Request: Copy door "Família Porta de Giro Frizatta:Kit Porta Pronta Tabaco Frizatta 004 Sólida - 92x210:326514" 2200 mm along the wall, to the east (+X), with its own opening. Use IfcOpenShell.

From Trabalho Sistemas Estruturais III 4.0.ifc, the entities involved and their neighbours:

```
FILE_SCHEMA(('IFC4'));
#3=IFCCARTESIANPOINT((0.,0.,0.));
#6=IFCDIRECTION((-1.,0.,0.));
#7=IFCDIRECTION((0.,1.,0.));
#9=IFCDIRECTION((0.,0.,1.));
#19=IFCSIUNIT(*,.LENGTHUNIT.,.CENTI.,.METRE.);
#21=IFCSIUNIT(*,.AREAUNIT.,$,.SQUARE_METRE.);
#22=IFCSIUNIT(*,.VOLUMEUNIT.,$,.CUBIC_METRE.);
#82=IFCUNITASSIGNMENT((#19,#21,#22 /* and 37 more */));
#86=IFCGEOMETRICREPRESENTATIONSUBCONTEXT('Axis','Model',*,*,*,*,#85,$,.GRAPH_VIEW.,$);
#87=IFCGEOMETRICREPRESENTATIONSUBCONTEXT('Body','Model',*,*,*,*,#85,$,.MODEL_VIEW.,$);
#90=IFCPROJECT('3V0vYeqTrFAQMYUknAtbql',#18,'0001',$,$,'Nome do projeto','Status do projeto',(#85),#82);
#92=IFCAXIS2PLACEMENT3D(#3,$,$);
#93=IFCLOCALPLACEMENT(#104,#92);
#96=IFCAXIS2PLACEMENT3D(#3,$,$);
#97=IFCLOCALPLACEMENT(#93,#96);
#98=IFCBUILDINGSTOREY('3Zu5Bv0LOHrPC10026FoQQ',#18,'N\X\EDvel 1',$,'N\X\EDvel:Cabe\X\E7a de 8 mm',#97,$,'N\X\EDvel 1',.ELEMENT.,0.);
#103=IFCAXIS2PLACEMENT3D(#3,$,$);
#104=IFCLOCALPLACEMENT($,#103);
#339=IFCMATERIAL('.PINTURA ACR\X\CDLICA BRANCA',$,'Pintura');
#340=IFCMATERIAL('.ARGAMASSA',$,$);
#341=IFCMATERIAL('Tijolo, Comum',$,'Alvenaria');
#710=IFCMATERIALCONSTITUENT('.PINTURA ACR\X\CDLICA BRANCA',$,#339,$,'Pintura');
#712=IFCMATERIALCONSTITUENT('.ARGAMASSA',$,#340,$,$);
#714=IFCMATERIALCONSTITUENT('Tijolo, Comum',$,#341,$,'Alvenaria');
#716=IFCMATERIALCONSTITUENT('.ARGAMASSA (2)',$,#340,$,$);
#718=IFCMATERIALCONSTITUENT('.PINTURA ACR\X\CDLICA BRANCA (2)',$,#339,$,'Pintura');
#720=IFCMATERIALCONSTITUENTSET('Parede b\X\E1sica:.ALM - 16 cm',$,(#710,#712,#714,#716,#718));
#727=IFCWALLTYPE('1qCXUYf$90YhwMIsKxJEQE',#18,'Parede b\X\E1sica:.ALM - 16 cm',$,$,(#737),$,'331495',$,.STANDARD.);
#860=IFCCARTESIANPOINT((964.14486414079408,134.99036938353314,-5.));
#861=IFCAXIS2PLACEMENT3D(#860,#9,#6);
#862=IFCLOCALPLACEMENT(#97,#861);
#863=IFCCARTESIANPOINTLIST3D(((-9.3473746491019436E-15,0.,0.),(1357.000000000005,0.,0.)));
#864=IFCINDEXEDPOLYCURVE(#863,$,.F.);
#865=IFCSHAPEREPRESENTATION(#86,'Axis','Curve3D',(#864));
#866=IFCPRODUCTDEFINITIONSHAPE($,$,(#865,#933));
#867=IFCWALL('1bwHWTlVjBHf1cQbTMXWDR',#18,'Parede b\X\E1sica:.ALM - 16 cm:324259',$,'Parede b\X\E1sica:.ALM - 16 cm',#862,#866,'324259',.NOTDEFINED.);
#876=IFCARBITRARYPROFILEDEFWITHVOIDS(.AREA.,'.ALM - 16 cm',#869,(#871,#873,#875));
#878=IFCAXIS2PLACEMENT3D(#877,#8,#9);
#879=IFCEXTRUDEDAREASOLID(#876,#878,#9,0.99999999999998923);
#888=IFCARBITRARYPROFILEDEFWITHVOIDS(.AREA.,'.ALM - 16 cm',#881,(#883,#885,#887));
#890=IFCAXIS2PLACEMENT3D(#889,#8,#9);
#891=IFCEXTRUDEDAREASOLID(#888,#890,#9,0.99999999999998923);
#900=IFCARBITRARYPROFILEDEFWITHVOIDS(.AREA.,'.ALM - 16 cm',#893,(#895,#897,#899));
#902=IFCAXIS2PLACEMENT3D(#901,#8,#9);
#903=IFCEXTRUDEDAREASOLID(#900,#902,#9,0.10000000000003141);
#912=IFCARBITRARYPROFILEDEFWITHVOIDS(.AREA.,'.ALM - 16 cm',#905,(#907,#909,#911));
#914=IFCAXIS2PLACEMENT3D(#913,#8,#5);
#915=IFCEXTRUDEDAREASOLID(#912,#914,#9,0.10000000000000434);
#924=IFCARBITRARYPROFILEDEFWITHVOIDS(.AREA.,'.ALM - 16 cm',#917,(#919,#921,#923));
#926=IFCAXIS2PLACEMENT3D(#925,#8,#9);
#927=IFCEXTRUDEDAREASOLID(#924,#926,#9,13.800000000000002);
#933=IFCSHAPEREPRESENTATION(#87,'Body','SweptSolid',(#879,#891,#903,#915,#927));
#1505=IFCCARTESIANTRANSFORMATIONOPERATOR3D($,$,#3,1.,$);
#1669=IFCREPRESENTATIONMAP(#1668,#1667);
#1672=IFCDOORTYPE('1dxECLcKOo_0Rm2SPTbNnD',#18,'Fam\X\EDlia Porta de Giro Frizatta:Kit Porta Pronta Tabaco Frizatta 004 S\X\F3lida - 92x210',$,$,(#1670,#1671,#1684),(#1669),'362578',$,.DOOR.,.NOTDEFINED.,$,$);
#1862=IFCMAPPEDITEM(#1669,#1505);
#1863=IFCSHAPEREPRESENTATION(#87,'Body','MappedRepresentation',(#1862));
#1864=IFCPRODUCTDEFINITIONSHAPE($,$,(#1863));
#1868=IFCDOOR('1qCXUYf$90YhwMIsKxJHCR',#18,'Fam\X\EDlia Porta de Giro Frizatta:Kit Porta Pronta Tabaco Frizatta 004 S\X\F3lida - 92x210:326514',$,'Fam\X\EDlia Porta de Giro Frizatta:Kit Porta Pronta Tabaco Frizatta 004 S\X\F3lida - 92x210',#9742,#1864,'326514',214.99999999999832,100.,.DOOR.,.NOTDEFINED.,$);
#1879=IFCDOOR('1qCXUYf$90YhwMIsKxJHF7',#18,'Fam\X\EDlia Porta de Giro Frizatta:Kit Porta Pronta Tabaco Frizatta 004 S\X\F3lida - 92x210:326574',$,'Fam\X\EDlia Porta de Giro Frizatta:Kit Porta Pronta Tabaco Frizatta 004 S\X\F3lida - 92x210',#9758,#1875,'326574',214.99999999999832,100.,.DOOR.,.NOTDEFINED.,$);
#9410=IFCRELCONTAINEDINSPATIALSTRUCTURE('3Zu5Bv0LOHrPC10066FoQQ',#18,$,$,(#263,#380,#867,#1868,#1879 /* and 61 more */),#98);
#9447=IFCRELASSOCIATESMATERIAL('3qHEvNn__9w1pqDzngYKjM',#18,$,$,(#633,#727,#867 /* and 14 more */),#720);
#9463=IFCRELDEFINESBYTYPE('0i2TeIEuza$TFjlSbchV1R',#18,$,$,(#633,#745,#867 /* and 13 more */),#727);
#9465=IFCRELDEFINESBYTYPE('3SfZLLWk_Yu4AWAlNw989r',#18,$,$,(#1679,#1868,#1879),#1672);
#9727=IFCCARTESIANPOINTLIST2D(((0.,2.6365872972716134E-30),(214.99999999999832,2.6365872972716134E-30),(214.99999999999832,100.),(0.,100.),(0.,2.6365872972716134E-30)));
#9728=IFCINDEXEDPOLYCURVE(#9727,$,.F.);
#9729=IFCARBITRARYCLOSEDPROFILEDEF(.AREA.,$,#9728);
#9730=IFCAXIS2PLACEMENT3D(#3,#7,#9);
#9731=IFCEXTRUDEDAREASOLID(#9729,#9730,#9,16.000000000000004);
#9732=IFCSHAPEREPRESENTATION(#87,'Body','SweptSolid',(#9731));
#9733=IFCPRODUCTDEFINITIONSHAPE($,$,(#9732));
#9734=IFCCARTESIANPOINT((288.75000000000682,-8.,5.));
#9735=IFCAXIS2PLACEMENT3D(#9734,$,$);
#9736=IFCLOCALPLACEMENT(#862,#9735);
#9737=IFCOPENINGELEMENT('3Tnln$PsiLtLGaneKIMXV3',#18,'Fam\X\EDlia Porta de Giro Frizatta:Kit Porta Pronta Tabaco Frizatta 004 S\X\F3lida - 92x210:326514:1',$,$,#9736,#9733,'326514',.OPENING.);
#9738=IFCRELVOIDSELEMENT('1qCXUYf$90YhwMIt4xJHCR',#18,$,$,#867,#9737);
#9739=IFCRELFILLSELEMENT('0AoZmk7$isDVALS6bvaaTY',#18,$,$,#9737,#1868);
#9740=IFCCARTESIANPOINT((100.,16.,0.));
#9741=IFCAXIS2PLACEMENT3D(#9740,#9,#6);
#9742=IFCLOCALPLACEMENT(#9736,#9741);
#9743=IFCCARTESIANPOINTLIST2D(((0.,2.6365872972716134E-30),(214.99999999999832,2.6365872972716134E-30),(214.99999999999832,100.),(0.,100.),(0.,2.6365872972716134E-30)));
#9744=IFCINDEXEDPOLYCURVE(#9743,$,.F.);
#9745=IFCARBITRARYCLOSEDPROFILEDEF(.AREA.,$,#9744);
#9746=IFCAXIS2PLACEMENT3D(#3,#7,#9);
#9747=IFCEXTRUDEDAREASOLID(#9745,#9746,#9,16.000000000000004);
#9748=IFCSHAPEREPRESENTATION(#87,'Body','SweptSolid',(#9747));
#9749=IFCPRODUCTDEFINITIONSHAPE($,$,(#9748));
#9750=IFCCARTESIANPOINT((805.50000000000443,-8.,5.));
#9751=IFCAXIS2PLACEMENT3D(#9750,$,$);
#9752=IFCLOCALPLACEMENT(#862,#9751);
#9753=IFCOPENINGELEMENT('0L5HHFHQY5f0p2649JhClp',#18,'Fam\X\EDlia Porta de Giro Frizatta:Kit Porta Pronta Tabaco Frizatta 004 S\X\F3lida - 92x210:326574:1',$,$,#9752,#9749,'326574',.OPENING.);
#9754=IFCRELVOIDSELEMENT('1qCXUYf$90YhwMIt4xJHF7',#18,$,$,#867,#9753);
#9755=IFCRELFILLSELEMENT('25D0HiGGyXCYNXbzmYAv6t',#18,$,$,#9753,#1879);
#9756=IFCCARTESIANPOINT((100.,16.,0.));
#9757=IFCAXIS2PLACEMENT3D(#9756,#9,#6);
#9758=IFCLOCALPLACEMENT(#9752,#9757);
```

```python
import ifcopenshell
import ifcopenshell.api.feature
import ifcopenshell.api.geometry
import ifcopenshell.api.root
import ifcopenshell.geom
import ifcopenshell.util.element
import ifcopenshell.util.placement
import ifcopenshell.util.shape
import ifcopenshell.util.unit

model = ifcopenshell.open("Trabalho Sistemas Estruturais III 4.0.ifc")
unit_scale = ifcopenshell.util.unit.calculate_unit_scale(model)
settings = ifcopenshell.geom.settings()


def volume(element):
    """Net volume in cubic metres, openings subtracted."""
    shape = ifcopenshell.geom.create_shape(settings, element)
    return ifcopenshell.util.shape.get_volume(shape.geometry)


def reuse_history(source, copy):
    """copy_class also copies each property set's owner history, people and application; keep the originals."""
    for rel in copy.IsDefinedBy:
        if rel.is_a("IfcRelDefinesByProperties") and (history := rel.RelatingPropertyDefinition.OwnerHistory):
            rel.RelatingPropertyDefinition.OwnerHistory = source.OwnerHistory
            ifcopenshell.util.element.remove_deep2(model, history)


door = model.by_guid("1qCXUYf$90YhwMIsKxJHCR")
opening = door.FillsVoids[0].RelatingOpeningElement
wall = opening.VoidsElements[0].RelatingBuildingElement
before = volume(wall)
shift = ifcopenshell.util.placement.get_local_placement(wall.ObjectPlacement)[:3, 0] * -2.2 / unit_scale

# copy_class copies the void relationship, type, container and properties, but no geometry.
new_opening = ifcopenshell.api.root.copy_class(model, product=opening)
new_opening.Representation = ifcopenshell.util.element.copy_deep(
    model, opening.Representation, exclude=["IfcGeometricRepresentationContext", "IfcRepresentationMap"]
)
new_opening.Name = "Família Porta de Giro Frizatta:Kit Porta Pronta Tabaco Frizatta 004 Sólida - 92x210"
new_opening.Tag = None
new_door = ifcopenshell.api.root.copy_class(model, product=door)
new_door.Representation = ifcopenshell.util.element.copy_deep(
    model, door.Representation, exclude=["IfcGeometricRepresentationContext", "IfcRepresentationMap"]
)
new_door.Name = "Família Porta de Giro Frizatta:Kit Porta Pronta Tabaco Frizatta 004 Sólida - 92x210"
new_door.Tag = None
reuse_history(door, new_door)
ifcopenshell.api.feature.add_filling(model, opening=new_opening, element=new_door)

for old, new in ((opening, new_opening), (door, new_door)):
    matrix = ifcopenshell.util.placement.get_local_placement(old.ObjectPlacement)
    matrix[:3, 3] += shift
    ifcopenshell.api.geometry.edit_object_placement(model, product=new, matrix=matrix, is_si=False)

after = volume(wall)

print(f"wall volume {before:.3f} -> {after:.3f} m3")

model.write("Trabalho Sistemas Estruturais III 4.0_updated.ifc")
```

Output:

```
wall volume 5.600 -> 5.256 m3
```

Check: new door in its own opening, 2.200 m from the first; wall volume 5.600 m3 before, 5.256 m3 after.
